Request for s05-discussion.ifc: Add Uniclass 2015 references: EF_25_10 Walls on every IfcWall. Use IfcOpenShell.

First a look at what the model holds.

```python
import ifcopenshell

model = ifcopenshell.open("s05-discussion.ifc")
print(model.schema)
print("classifications:", [c.Name for c in model.by_type("IfcClassification")])
for ifc_class in ("IfcDoor", "IfcRoof", "IfcStair", "IfcWall", "IfcWindow"):
    print(ifc_class, len(model.by_type(ifc_class)))
```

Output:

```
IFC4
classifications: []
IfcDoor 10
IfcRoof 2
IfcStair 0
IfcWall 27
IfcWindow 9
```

```python
import ifcopenshell
import ifcopenshell.api.classification

model = ifcopenshell.open("s05-discussion.ifc")

system = ifcopenshell.api.classification.add_classification(model, classification="Uniclass 2015")

codes = {
    "IfcWall": ("EF_25_10", "Walls"),
}
for ifc_class, (code, name) in codes.items():
    products = model.by_type(ifc_class)
    ifcopenshell.api.classification.add_reference(
        model, products=products, classification=system, identification=code, name=name
    )
    print(code, len(products))

model.write("s05-discussion-out.ifc")
```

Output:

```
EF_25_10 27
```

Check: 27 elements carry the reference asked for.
